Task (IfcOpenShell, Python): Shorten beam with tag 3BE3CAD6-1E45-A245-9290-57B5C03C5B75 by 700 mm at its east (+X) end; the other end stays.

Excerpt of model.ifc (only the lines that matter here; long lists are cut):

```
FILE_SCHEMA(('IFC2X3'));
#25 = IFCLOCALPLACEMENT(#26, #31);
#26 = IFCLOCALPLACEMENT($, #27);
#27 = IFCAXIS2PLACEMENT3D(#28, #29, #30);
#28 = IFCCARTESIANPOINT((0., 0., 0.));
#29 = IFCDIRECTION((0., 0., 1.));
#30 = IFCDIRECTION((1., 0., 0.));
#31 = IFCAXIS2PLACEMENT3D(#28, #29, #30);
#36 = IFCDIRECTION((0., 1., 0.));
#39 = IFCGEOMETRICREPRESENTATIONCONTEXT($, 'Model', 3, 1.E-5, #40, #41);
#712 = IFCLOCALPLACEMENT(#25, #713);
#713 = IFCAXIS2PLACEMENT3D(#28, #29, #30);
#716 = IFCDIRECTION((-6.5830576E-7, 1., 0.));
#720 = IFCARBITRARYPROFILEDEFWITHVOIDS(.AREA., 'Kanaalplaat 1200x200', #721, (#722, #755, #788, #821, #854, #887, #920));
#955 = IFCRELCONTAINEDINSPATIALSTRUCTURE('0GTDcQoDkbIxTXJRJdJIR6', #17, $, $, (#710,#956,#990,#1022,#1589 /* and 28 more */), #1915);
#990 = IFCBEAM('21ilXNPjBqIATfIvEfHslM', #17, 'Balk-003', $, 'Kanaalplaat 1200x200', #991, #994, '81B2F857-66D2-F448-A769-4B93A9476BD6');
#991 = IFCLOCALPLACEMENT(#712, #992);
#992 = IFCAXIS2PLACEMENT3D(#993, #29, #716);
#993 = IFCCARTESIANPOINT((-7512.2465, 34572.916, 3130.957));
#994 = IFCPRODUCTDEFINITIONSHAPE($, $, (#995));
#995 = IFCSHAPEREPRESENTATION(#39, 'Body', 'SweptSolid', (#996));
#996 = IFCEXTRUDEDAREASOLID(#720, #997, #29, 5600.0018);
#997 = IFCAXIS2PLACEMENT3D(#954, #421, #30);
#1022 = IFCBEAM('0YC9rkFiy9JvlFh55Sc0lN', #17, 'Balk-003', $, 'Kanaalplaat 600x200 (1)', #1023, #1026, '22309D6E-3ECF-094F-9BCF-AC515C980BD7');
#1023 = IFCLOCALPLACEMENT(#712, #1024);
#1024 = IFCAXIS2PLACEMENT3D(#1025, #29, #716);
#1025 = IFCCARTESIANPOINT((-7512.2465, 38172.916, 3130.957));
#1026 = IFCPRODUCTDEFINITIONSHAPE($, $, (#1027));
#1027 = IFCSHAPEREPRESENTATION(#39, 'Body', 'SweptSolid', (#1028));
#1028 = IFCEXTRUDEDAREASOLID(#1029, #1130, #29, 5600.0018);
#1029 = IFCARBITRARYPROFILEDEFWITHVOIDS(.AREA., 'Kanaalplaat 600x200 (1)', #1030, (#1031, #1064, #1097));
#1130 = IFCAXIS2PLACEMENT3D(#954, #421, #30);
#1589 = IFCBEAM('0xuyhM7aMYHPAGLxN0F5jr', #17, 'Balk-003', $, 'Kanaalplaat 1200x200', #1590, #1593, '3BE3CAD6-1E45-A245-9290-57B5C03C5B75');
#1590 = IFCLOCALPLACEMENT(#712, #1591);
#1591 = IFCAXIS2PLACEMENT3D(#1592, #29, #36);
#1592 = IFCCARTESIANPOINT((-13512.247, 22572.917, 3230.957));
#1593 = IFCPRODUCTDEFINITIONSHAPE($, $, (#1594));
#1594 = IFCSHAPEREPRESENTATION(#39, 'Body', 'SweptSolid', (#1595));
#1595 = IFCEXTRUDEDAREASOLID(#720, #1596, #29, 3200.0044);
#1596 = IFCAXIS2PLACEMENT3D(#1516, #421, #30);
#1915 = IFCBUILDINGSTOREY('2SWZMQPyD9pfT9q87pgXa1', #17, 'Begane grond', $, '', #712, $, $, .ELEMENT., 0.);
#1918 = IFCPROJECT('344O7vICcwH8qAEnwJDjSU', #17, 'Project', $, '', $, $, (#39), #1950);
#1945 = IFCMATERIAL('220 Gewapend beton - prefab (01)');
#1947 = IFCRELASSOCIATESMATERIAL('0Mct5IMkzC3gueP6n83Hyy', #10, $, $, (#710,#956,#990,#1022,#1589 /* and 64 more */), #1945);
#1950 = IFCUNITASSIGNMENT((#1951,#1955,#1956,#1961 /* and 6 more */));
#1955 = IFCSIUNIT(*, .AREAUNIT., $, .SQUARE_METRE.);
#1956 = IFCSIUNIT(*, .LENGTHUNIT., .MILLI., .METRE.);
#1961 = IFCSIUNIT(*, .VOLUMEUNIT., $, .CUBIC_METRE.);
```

```python
import ifcopenshell
import ifcopenshell.util.unit

model = ifcopenshell.open("model.ifc")
unit_scale = ifcopenshell.util.unit.calculate_unit_scale(model)

member = model.by_id(1589)
change = -0.7 / unit_scale

# The extrusion runs towards the end named, so only its depth changes.
body = next(r for r in member.Representation.Representations if r.RepresentationIdentifier == "Body")
solid = body.Items[0]
old_length = solid.Depth
solid.Depth += change

print(f"length {old_length:g} -> {solid.Depth:g}")

model.write("model_rev.ifc")
```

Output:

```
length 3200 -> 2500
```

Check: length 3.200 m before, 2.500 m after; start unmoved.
